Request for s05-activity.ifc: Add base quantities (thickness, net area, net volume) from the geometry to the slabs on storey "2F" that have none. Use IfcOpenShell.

First a look at what the model holds.

```python
import ifcopenshell
import ifcopenshell.util.element
import ifcopenshell.util.unit

model = ifcopenshell.open("s05-activity.ifc")
print(model.schema)
for unit_type in ("LENGTHUNIT", "AREAUNIT", "VOLUMEUNIT"):
    print(unit_type, ifcopenshell.util.unit.calculate_unit_scale(model, unit_type))
storey = next(s for s in model.by_type("IfcBuildingStorey") if s.Name == "2F")
slabs = [e for e in ifcopenshell.util.element.get_decomposition(storey) if e.is_a("IfcSlab")]
for e in sorted(slabs, key=lambda e: e.id()):
    print(e.id(), e.is_a(), e.Name, list(ifcopenshell.util.element.get_psets(e, qtos_only=True)), sep=" | ")
```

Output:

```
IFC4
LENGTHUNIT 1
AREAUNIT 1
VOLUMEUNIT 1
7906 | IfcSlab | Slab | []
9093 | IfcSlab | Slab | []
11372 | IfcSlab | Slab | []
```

```python
import ifcopenshell
import ifcopenshell.api.pset
import ifcopenshell.geom
import ifcopenshell.util.element
import ifcopenshell.util.shape
import ifcopenshell.util.unit

model = ifcopenshell.open("s05-activity.ifc")
unit_scale = ifcopenshell.util.unit.calculate_unit_scale(model)
area_scale = ifcopenshell.util.unit.calculate_unit_scale(model, "AREAUNIT")
volume_scale = ifcopenshell.util.unit.calculate_unit_scale(model, "VOLUMEUNIT")
settings = ifcopenshell.geom.settings()

storey = next(s for s in model.by_type("IfcBuildingStorey") if s.Name == "2F")
slabs = [e for e in ifcopenshell.util.element.get_decomposition(storey) if e.is_a("IfcSlab")]

for e in sorted(slabs, key=lambda e: e.id()):
    if ifcopenshell.util.element.get_psets(e, qtos_only=True, should_inherit=False):
        continue
    # Geometry comes back in metres, in the element's own axes.
    shape = ifcopenshell.geom.create_shape(settings, e)
    values = {
        "Width": ifcopenshell.util.shape.get_z(shape.geometry) / unit_scale,
        "NetArea": ifcopenshell.util.shape.get_footprint_area(shape.geometry) / area_scale,
        "NetVolume": ifcopenshell.util.shape.get_volume(shape.geometry) / volume_scale,
    }
    qto = ifcopenshell.api.pset.add_qto(model, product=e, name="Qto_SlabBaseQuantities")
    ifcopenshell.api.pset.edit_qto(model, qto=qto, properties=values)
    print(e.id(), {k: round(v, 3) for k, v in values.items()})

model.write("s05-activity-out.ifc")
```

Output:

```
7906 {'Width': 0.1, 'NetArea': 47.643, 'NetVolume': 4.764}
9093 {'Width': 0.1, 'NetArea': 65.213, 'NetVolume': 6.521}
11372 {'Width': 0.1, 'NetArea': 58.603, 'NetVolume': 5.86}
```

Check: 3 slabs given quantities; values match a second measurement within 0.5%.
